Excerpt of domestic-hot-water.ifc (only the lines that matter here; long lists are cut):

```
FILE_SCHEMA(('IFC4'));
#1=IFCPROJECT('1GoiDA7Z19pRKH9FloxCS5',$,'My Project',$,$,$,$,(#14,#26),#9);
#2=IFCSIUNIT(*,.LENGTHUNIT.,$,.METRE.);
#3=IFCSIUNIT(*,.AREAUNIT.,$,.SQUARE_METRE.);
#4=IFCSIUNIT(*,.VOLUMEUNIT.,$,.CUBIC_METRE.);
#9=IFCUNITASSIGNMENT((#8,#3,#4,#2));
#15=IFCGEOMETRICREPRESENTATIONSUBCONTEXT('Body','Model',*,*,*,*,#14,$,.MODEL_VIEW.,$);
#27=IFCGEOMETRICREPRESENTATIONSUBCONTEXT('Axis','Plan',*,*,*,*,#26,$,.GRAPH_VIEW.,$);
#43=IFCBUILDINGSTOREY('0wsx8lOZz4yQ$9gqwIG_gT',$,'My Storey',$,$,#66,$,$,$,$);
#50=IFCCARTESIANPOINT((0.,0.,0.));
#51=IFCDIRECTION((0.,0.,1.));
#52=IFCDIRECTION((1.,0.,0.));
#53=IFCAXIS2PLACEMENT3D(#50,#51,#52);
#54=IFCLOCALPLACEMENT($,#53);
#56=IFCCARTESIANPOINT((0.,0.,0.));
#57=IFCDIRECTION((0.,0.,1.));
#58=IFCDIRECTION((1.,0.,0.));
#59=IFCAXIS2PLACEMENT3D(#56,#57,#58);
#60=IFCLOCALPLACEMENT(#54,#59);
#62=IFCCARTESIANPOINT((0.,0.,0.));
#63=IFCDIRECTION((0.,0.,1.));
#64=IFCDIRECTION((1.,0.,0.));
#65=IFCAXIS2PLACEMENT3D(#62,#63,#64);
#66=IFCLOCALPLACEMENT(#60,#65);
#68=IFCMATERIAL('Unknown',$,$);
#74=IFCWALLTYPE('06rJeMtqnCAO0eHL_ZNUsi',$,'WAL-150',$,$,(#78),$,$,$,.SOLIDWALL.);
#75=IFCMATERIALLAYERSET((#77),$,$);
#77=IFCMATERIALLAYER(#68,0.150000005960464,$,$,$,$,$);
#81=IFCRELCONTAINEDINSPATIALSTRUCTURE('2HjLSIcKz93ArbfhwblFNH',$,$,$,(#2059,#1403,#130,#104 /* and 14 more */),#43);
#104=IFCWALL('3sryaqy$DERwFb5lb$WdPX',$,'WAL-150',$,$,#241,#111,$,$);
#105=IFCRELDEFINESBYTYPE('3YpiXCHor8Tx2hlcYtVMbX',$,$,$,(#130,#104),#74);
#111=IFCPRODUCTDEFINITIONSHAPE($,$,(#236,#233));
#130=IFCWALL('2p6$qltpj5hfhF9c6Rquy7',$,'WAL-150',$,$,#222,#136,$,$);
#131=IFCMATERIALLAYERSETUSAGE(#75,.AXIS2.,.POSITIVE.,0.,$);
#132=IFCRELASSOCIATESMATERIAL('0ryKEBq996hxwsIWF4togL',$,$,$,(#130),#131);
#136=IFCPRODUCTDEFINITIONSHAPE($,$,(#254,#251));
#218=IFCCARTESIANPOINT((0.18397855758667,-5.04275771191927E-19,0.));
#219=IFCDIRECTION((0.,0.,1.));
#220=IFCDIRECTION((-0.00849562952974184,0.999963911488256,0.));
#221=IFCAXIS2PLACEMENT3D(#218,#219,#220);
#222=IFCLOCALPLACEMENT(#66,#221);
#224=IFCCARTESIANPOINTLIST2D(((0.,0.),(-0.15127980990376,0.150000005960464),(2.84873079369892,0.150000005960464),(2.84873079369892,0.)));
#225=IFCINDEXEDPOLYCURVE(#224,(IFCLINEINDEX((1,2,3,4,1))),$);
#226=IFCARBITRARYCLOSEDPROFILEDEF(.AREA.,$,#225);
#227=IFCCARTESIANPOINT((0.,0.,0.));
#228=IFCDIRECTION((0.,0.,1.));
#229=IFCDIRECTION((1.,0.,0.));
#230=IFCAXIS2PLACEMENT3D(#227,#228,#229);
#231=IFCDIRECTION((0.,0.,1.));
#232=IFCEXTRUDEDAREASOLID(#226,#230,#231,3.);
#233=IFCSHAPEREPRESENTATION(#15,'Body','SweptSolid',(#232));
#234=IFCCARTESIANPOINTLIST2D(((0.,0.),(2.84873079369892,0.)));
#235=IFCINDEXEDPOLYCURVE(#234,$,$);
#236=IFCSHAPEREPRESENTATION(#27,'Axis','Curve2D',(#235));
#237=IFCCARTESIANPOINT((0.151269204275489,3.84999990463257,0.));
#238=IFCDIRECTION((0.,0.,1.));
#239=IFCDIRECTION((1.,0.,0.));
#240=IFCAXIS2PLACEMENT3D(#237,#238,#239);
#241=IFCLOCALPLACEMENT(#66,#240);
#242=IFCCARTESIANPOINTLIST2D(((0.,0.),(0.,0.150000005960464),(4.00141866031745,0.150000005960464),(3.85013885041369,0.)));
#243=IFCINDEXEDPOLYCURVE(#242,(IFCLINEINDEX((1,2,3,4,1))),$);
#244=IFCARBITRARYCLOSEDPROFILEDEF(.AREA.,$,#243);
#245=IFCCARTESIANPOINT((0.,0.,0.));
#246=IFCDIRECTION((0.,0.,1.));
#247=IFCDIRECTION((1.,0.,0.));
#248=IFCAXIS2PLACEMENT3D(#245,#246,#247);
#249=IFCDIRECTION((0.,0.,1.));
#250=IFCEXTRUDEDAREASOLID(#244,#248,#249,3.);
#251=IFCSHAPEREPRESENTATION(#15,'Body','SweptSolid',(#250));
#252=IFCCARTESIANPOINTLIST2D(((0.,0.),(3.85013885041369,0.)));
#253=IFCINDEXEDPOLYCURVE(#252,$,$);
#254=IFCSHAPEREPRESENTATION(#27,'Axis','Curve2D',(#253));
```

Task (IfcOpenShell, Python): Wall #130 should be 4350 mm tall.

```python
import ifcopenshell
import ifcopenshell.geom
import ifcopenshell.util.representation
import ifcopenshell.util.shape
import ifcopenshell.util.unit

model = ifcopenshell.open("domestic-hot-water.ifc")
unit_scale = ifcopenshell.util.unit.calculate_unit_scale(model)
settings = ifcopenshell.geom.settings()


def volume(element):
    """Net volume in cubic metres, openings subtracted."""
    shape = ifcopenshell.geom.create_shape(settings, element)
    return ifcopenshell.util.shape.get_volume(shape.geometry)


wall = model.by_guid("2p6$qltpj5hfhF9c6Rquy7")
before = volume(wall)

body = ifcopenshell.util.representation.get_representation(wall, "Model", "Body")
solid = body.Items[0]
old_height = solid.Depth
solid.Depth = 4.35 / unit_scale
after = volume(wall)

print(f"height {old_height:g} -> {solid.Depth:g}, volume {before:.3f} -> {after:.3f} m3")

model.write("domestic-hot-water_edited.ifc")
```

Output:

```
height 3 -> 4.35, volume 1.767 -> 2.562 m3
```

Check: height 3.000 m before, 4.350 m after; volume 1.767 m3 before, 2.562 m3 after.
